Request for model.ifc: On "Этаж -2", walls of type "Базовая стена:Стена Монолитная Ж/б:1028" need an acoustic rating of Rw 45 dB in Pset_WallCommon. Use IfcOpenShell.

First a look at what the model holds.

```python
import ifcopenshell
import ifcopenshell.util.element

model = ifcopenshell.open("model.ifc")
print(model.schema)
storey = next(s for s in model.by_type("IfcBuildingStorey") if s.Name == "Этаж -2")
walls = [e for e in ifcopenshell.util.element.get_decomposition(storey) if e.is_a("IfcWall")]
seen = {}
for e in walls:
    element_type = ifcopenshell.util.element.get_type(e)
    key = (element_type.Name if element_type != e and element_type else None, ifcopenshell.util.element.get_pset(e, "Pset_WallCommon", "AcousticRating"))
    seen[key] = seen.get(key, 0) + 1
for (name, value), count in sorted(seen.items(), key=str):
    print(count, "x", name, "|", value)
```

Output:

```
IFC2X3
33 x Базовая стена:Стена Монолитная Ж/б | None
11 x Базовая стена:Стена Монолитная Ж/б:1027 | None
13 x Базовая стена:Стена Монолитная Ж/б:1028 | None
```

```python
import ifcopenshell
import ifcopenshell.api.pset
import ifcopenshell.util.element

model = ifcopenshell.open("model.ifc")

storey = next(s for s in model.by_type("IfcBuildingStorey") if s.Name == "Этаж -2")
walls = [e for e in ifcopenshell.util.element.get_decomposition(storey) if e.is_a("IfcWall")]

count = 0
for e in walls:
    element_type = ifcopenshell.util.element.get_type(e)
    if element_type in (None, e) or element_type.Name != "Базовая стена:Стена Монолитная Ж/б:1028":
        continue
    # add_pset returns the element's existing set when there is one.
    pset = ifcopenshell.api.pset.add_pset(model, product=e, name="Pset_WallCommon")
    ifcopenshell.api.pset.edit_pset(model, pset=pset, properties={"AcousticRating": "Rw 45 dB"})
    count += 1

print(count, "walls updated")

model.write("model_updated.ifc")
```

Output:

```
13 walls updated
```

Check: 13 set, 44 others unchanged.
